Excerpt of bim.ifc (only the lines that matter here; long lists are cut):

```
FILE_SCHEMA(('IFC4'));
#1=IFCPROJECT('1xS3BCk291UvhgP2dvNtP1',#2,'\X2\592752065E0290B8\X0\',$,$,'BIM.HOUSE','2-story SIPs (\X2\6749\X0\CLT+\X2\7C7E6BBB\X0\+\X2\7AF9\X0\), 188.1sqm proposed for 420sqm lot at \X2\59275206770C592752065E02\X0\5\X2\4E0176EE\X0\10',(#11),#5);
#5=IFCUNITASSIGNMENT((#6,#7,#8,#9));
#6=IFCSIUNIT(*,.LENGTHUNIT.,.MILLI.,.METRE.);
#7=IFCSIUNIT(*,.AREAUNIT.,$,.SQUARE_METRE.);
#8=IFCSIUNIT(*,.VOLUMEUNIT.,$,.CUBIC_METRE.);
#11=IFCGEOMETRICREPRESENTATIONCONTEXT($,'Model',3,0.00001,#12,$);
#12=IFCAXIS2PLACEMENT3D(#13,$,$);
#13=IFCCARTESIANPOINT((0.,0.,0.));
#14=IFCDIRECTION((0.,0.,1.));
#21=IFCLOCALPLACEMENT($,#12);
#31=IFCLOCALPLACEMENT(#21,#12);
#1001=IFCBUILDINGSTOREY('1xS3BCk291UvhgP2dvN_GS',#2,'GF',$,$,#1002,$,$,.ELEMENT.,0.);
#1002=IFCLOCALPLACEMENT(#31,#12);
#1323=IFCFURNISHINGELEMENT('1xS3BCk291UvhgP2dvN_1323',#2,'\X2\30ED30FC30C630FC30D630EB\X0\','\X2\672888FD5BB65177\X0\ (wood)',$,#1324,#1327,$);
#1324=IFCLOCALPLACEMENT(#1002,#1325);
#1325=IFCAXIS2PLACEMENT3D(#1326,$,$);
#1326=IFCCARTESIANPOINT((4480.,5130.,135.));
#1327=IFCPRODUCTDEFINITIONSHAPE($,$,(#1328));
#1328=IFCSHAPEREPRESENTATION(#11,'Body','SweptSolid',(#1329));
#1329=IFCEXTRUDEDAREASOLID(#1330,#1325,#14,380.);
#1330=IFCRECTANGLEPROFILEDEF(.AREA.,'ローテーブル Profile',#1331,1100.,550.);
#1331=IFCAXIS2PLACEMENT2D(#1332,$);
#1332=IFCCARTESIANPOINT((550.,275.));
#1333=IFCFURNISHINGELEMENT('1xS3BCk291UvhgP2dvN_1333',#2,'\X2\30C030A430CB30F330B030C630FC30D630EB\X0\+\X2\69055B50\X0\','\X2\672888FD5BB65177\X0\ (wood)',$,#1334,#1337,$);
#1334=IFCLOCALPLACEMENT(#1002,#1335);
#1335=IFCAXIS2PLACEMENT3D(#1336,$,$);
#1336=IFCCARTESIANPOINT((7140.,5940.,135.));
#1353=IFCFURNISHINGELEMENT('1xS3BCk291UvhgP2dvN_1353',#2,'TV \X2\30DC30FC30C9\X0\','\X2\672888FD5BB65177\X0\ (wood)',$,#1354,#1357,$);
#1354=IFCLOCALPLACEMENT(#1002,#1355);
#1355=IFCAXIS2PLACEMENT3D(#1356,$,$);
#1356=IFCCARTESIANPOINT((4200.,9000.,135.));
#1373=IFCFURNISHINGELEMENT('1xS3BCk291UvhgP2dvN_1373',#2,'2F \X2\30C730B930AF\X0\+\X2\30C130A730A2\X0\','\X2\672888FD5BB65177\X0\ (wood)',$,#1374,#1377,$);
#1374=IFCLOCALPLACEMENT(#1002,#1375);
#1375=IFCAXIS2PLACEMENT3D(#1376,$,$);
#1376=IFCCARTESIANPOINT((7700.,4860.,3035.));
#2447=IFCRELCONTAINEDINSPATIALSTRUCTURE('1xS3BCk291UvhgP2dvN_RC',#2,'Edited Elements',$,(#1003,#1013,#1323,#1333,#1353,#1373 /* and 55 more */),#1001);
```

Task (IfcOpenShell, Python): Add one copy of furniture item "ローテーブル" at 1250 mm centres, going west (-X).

```python
import numpy as np
import ifcopenshell
import ifcopenshell.api.geometry
import ifcopenshell.api.root
import ifcopenshell.util.element
import ifcopenshell.util.placement
import ifcopenshell.util.unit

model = ifcopenshell.open("bim.ifc")
unit_scale = ifcopenshell.util.unit.calculate_unit_scale(model)


def reuse_history(source, copy):
    """copy_class also copies each property set's owner history, people and application; keep the originals."""
    for rel in copy.IsDefinedBy:
        if rel.is_a("IfcRelDefinesByProperties") and (history := rel.RelatingPropertyDefinition.OwnerHistory):
            rel.RelatingPropertyDefinition.OwnerHistory = source.OwnerHistory
            ifcopenshell.util.element.remove_deep2(model, history)


source = model.by_guid("1xS3BCk291UvhgP2dvN_1323")
base = ifcopenshell.util.placement.get_local_placement(source.ObjectPlacement)
step = np.array([-1.0, 0.0, 0.0]) * 1.25 / unit_scale

for i in range(1, 2):
    copy = ifcopenshell.api.root.copy_class(model, product=source)
    copy.Representation = ifcopenshell.util.element.copy_deep(
        model, source.Representation, exclude=["IfcGeometricRepresentationContext", "IfcRepresentationMap"]
    )
    reuse_history(source, copy)
    matrix = base.copy()
    matrix[:3, 3] += i * step
    print("added at", matrix[:3, 3].round(3) + 0.0)
    ifcopenshell.api.geometry.edit_object_placement(model, product=copy, matrix=matrix, is_si=False)

model.write("bim_updated.ifc")
```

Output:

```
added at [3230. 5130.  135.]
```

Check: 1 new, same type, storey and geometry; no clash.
